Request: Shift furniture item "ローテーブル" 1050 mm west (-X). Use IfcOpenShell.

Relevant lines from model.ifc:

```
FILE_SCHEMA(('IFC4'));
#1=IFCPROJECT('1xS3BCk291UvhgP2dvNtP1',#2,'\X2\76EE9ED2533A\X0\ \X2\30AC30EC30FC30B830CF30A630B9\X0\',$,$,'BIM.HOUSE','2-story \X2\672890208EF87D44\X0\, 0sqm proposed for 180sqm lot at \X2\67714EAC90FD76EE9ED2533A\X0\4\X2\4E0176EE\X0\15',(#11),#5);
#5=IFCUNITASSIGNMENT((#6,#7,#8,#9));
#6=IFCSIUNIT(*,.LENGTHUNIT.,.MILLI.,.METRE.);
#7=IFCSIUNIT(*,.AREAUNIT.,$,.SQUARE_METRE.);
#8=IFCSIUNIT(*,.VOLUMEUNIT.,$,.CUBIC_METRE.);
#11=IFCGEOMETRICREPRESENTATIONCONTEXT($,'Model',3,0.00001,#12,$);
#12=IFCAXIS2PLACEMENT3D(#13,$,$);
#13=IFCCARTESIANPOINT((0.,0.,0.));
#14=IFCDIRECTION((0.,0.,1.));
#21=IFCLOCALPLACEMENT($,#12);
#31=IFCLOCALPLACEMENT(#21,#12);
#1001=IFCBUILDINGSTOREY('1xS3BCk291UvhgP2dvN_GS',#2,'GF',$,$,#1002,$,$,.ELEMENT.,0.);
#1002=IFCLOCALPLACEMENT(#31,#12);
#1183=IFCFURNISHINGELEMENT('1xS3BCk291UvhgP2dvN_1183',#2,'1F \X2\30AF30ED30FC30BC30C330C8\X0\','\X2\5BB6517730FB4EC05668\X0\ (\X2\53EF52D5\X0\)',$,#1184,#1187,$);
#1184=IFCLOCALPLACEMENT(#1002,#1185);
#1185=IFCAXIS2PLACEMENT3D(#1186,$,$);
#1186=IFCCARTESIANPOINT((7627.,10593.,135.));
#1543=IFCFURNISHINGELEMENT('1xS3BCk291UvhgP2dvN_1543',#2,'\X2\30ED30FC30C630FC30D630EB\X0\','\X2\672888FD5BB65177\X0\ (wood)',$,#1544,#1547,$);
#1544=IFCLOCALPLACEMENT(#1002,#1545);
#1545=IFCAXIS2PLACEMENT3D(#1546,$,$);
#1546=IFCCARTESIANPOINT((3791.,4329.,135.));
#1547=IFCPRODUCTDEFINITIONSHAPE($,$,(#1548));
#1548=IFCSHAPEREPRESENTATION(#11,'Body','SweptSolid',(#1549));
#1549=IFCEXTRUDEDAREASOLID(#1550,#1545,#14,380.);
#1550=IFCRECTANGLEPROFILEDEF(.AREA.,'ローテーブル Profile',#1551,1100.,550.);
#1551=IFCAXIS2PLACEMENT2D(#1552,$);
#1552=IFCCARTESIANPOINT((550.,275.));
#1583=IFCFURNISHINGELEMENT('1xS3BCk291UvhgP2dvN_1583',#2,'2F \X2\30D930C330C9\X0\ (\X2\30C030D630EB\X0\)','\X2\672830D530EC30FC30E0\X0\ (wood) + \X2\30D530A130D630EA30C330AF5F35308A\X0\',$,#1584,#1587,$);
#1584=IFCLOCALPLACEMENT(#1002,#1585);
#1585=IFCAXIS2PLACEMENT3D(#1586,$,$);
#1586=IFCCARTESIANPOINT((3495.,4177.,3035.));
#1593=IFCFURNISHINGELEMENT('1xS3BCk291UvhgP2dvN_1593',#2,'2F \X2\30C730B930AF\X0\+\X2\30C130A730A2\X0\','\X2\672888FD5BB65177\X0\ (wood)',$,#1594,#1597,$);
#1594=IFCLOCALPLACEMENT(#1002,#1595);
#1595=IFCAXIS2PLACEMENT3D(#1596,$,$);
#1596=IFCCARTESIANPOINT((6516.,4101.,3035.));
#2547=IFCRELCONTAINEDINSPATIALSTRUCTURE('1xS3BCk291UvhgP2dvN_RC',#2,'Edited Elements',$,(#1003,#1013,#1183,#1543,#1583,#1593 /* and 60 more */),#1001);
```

```python
import ifcopenshell
import ifcopenshell.api.geometry
import ifcopenshell.util.placement

model = ifcopenshell.open("model.ifc")

item = model.by_guid("1xS3BCk291UvhgP2dvN_1543")
matrix = ifcopenshell.util.placement.get_local_placement(item.ObjectPlacement)
matrix[0, 3] -= 1050.0
ifcopenshell.api.geometry.edit_object_placement(model, product=item, matrix=matrix, is_si=False)

print(ifcopenshell.util.placement.get_local_placement(item.ObjectPlacement).round(3) + 0.0)

model.write("model_updated.ifc")
```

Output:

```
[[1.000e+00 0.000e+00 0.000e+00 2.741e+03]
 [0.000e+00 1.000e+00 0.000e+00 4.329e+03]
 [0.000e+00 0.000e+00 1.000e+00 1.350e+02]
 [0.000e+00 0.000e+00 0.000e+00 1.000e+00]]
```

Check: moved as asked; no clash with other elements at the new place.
